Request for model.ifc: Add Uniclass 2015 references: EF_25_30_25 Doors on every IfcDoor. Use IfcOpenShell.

First a look at what the model holds.

```python
import ifcopenshell

model = ifcopenshell.open("model.ifc")
print(model.schema)
print("classifications:", [c.Name for c in model.by_type("IfcClassification")])
for ifc_class in ("IfcDoor", "IfcRoof", "IfcStair", "IfcWall", "IfcWindow"):
    print(ifc_class, len(model.by_type(ifc_class)))
```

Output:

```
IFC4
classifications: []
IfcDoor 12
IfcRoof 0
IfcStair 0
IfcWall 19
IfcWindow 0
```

```python
import ifcopenshell
import ifcopenshell.api.classification

model = ifcopenshell.open("model.ifc")

system = ifcopenshell.api.classification.add_classification(model, classification="Uniclass 2015")

codes = {
    "IfcDoor": ("EF_25_30_25", "Doors"),
}
for ifc_class, (code, name) in codes.items():
    products = model.by_type(ifc_class)
    ifcopenshell.api.classification.add_reference(
        model, products=products, classification=system, identification=code, name=name
    )
    print(code, len(products))

model.write("model-out.ifc")
```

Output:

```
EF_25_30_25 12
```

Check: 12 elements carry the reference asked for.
